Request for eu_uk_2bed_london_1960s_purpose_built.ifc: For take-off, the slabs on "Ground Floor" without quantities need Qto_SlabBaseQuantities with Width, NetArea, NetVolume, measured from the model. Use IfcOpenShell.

First a look at what the model holds.

```python
import ifcopenshell
import ifcopenshell.util.element
import ifcopenshell.util.unit

model = ifcopenshell.open("eu_uk_2bed_london_1960s_purpose_built.ifc")
print(model.schema)
for unit_type in ("LENGTHUNIT", "AREAUNIT", "VOLUMEUNIT"):
    print(unit_type, ifcopenshell.util.unit.calculate_unit_scale(model, unit_type))
storey = next(s for s in model.by_type("IfcBuildingStorey") if s.Name == "Ground Floor")
slabs = [e for e in ifcopenshell.util.element.get_decomposition(storey) if e.is_a("IfcSlab")]
for e in sorted(slabs, key=lambda e: e.id()):
    print(e.id(), e.is_a(), e.Name, list(ifcopenshell.util.element.get_psets(e, qtos_only=True)), sep=" | ")
```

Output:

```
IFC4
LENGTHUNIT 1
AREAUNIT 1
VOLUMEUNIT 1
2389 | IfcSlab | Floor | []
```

```python
import ifcopenshell
import ifcopenshell.api.pset
import ifcopenshell.geom
import ifcopenshell.util.element
import ifcopenshell.util.shape
import ifcopenshell.util.unit

model = ifcopenshell.open("eu_uk_2bed_london_1960s_purpose_built.ifc")
unit_scale = ifcopenshell.util.unit.calculate_unit_scale(model)
area_scale = ifcopenshell.util.unit.calculate_unit_scale(model, "AREAUNIT")
volume_scale = ifcopenshell.util.unit.calculate_unit_scale(model, "VOLUMEUNIT")
settings = ifcopenshell.geom.settings()

storey = next(s for s in model.by_type("IfcBuildingStorey") if s.Name == "Ground Floor")
slabs = [e for e in ifcopenshell.util.element.get_decomposition(storey) if e.is_a("IfcSlab")]

for e in sorted(slabs, key=lambda e: e.id()):
    if ifcopenshell.util.element.get_psets(e, qtos_only=True, should_inherit=False):
        continue
    # Geometry comes back in metres, in the element's own axes.
    shape = ifcopenshell.geom.create_shape(settings, e)
    values = {
        "Width": ifcopenshell.util.shape.get_z(shape.geometry) / unit_scale,
        "NetArea": ifcopenshell.util.shape.get_footprint_area(shape.geometry) / area_scale,
        "NetVolume": ifcopenshell.util.shape.get_volume(shape.geometry) / volume_scale,
    }
    qto = ifcopenshell.api.pset.add_qto(model, product=e, name="Qto_SlabBaseQuantities")
    ifcopenshell.api.pset.edit_qto(model, qto=qto, properties=values)
    print(e.id(), {k: round(v, 3) for k, v in values.items()})

model.write("eu_uk_2bed_london_1960s_purpose_built_rev.ifc")
```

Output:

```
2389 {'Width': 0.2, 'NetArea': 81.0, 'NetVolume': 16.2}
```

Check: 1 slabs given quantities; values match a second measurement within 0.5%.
